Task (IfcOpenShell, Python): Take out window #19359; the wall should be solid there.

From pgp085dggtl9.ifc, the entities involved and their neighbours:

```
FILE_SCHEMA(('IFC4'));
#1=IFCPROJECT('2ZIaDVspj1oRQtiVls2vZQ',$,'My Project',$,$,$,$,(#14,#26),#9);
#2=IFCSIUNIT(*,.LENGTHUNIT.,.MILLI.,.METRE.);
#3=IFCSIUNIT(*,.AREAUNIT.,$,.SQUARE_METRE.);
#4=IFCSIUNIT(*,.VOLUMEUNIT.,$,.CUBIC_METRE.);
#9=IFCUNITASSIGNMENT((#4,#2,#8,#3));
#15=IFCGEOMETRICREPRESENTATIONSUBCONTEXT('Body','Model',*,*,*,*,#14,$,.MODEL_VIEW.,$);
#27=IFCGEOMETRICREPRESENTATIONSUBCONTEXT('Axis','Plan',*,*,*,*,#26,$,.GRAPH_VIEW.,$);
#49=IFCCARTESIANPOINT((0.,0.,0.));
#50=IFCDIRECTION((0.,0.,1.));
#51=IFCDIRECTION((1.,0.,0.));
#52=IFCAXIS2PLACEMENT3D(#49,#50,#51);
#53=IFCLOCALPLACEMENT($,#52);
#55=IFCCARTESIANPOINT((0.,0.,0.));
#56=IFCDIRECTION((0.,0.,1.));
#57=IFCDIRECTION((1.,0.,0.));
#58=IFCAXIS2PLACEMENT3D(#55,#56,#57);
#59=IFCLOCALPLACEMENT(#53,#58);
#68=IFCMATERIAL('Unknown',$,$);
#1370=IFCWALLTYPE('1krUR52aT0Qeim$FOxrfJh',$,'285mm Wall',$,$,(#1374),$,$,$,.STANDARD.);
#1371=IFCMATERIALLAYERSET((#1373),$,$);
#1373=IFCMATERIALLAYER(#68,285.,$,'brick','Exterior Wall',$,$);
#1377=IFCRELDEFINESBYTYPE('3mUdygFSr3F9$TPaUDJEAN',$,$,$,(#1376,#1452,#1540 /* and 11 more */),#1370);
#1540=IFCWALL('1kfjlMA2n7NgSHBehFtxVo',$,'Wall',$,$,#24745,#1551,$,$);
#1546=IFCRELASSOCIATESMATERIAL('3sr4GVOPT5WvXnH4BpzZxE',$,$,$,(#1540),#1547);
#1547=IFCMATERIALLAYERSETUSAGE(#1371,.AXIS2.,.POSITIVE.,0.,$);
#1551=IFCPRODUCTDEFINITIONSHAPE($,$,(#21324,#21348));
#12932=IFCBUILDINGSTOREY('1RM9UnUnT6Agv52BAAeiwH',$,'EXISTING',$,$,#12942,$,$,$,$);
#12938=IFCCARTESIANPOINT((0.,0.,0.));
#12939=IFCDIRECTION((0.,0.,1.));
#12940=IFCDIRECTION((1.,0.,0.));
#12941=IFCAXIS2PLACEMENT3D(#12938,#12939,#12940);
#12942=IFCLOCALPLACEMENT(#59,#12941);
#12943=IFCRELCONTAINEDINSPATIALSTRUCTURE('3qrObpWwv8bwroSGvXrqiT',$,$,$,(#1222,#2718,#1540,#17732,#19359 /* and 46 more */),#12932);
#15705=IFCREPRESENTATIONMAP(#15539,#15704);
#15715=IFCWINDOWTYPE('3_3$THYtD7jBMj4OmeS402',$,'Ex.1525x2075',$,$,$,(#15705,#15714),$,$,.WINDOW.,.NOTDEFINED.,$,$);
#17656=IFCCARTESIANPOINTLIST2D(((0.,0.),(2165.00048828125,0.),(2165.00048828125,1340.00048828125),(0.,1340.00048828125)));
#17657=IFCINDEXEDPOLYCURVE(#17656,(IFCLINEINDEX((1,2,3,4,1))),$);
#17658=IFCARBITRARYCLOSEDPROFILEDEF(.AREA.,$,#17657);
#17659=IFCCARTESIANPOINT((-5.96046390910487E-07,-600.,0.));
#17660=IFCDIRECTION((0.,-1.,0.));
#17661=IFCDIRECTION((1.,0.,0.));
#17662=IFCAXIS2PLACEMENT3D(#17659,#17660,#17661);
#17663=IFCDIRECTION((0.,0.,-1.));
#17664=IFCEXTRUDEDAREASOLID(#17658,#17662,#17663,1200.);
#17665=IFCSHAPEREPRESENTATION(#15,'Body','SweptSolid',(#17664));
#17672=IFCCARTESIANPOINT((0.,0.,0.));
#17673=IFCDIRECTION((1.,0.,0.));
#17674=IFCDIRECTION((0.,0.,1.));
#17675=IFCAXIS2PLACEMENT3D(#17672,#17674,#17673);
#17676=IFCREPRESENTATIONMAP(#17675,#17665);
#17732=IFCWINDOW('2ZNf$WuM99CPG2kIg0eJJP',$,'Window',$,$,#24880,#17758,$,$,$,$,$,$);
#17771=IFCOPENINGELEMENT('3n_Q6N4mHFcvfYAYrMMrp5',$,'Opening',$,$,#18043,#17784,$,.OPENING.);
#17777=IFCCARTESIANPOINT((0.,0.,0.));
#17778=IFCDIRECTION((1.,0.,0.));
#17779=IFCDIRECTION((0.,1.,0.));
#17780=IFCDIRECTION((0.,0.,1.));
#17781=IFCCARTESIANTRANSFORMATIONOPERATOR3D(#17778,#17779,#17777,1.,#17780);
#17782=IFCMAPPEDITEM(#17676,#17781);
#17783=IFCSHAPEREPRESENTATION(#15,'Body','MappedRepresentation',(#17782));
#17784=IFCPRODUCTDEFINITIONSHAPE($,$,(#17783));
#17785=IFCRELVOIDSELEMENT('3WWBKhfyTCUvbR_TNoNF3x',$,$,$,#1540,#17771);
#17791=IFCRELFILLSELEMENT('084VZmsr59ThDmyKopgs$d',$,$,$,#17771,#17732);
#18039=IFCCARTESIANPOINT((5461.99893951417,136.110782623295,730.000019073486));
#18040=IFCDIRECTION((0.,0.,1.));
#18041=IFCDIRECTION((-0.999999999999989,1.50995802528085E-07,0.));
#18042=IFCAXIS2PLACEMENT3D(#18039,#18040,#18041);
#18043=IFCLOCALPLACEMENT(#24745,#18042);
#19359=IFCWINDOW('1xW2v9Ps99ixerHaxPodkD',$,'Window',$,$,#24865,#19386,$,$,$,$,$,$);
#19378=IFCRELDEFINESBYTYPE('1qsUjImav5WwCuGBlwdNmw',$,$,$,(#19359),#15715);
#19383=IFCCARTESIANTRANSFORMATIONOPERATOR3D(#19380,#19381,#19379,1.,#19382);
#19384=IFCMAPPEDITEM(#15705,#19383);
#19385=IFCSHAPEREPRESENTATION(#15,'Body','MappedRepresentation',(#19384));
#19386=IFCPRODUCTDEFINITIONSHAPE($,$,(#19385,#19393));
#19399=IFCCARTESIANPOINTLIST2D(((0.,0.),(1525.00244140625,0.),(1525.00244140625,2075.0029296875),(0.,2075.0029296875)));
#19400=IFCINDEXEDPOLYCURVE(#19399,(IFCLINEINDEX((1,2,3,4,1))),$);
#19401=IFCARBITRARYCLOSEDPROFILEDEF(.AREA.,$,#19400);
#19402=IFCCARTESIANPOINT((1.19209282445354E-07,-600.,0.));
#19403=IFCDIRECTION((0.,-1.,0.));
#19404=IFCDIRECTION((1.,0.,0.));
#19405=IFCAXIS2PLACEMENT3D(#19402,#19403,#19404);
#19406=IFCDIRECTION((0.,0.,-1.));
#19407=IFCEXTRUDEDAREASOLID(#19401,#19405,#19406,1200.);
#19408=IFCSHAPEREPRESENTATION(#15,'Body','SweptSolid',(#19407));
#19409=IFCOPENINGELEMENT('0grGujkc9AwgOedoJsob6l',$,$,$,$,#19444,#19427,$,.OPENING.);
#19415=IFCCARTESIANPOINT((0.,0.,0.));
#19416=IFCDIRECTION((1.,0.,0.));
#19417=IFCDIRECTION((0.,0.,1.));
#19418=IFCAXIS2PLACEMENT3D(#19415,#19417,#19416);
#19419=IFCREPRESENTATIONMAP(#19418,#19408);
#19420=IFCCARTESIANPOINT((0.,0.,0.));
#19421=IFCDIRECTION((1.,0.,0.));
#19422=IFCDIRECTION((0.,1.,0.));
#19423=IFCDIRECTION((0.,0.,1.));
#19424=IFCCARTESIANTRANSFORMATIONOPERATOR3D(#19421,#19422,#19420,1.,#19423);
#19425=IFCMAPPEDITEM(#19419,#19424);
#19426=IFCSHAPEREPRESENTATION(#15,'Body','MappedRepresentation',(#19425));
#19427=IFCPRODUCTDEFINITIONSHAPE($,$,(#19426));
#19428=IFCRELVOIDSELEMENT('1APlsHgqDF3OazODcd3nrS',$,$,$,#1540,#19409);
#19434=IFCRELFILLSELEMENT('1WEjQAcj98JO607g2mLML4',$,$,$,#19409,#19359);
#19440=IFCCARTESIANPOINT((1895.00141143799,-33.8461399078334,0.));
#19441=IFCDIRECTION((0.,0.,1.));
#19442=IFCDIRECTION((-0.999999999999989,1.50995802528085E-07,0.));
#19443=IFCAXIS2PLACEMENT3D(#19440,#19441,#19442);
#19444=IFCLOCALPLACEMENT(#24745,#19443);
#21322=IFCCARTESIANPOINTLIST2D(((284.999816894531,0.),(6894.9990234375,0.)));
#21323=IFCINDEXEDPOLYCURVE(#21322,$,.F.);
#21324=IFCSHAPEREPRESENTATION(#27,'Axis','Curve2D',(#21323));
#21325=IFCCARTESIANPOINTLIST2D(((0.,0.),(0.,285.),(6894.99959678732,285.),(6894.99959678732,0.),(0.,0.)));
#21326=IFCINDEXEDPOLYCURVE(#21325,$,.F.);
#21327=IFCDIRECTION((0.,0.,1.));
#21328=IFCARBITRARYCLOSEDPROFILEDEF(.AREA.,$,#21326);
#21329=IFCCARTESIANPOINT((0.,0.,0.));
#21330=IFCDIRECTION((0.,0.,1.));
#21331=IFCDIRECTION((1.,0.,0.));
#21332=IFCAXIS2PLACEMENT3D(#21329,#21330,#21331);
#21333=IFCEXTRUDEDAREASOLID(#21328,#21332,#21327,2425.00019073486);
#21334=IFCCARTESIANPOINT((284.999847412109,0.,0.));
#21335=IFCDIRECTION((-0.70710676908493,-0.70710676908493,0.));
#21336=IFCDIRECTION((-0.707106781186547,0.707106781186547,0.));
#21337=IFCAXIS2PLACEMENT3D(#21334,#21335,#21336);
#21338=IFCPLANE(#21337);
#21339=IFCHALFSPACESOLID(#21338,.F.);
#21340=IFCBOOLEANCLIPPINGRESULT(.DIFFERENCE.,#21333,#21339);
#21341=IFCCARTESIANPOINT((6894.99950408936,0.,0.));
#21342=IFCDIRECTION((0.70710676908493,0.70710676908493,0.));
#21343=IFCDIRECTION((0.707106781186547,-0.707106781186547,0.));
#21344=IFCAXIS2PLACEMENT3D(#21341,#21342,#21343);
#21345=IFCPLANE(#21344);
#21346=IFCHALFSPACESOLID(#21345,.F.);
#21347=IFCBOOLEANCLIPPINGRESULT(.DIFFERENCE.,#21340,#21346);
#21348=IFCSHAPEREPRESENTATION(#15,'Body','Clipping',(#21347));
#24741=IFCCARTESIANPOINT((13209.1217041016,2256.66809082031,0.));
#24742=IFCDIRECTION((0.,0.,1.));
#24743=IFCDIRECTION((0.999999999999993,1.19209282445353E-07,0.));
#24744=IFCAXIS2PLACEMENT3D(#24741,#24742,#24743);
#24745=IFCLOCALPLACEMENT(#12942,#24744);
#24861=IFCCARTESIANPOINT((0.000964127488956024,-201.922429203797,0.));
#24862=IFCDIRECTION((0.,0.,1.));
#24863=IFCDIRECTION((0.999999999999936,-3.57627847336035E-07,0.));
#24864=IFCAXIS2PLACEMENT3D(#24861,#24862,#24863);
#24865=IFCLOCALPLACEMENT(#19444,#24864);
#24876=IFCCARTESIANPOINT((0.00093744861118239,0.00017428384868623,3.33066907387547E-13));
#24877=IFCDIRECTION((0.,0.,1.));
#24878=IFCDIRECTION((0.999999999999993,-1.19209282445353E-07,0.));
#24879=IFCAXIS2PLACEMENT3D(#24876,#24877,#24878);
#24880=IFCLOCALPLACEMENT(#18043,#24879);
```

```python
import ifcopenshell
import ifcopenshell.api.feature
import ifcopenshell.api.root
import ifcopenshell.geom
import ifcopenshell.util.shape

model = ifcopenshell.open("pgp085dggtl9.ifc")
settings = ifcopenshell.geom.settings()


def volume(element):
    """Net volume in cubic metres, openings subtracted."""
    shape = ifcopenshell.geom.create_shape(settings, element)
    return ifcopenshell.util.shape.get_volume(shape.geometry)


window = model.by_guid("1xW2v9Ps99ixerHaxPodkD")
opening = window.FillsVoids[0].RelatingOpeningElement
wall = opening.VoidsElements[0].RelatingBuildingElement
before = volume(wall)

ifcopenshell.api.root.remove_product(model, product=window)
ifcopenshell.api.feature.remove_feature(model, feature=opening)

after = volume(wall)

print(f"wall volume {before:.3f} -> {after:.3f} m3")

model.write("pgp085dggtl9-out.ifc")
```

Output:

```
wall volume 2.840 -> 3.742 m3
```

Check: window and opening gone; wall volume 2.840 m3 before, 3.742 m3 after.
